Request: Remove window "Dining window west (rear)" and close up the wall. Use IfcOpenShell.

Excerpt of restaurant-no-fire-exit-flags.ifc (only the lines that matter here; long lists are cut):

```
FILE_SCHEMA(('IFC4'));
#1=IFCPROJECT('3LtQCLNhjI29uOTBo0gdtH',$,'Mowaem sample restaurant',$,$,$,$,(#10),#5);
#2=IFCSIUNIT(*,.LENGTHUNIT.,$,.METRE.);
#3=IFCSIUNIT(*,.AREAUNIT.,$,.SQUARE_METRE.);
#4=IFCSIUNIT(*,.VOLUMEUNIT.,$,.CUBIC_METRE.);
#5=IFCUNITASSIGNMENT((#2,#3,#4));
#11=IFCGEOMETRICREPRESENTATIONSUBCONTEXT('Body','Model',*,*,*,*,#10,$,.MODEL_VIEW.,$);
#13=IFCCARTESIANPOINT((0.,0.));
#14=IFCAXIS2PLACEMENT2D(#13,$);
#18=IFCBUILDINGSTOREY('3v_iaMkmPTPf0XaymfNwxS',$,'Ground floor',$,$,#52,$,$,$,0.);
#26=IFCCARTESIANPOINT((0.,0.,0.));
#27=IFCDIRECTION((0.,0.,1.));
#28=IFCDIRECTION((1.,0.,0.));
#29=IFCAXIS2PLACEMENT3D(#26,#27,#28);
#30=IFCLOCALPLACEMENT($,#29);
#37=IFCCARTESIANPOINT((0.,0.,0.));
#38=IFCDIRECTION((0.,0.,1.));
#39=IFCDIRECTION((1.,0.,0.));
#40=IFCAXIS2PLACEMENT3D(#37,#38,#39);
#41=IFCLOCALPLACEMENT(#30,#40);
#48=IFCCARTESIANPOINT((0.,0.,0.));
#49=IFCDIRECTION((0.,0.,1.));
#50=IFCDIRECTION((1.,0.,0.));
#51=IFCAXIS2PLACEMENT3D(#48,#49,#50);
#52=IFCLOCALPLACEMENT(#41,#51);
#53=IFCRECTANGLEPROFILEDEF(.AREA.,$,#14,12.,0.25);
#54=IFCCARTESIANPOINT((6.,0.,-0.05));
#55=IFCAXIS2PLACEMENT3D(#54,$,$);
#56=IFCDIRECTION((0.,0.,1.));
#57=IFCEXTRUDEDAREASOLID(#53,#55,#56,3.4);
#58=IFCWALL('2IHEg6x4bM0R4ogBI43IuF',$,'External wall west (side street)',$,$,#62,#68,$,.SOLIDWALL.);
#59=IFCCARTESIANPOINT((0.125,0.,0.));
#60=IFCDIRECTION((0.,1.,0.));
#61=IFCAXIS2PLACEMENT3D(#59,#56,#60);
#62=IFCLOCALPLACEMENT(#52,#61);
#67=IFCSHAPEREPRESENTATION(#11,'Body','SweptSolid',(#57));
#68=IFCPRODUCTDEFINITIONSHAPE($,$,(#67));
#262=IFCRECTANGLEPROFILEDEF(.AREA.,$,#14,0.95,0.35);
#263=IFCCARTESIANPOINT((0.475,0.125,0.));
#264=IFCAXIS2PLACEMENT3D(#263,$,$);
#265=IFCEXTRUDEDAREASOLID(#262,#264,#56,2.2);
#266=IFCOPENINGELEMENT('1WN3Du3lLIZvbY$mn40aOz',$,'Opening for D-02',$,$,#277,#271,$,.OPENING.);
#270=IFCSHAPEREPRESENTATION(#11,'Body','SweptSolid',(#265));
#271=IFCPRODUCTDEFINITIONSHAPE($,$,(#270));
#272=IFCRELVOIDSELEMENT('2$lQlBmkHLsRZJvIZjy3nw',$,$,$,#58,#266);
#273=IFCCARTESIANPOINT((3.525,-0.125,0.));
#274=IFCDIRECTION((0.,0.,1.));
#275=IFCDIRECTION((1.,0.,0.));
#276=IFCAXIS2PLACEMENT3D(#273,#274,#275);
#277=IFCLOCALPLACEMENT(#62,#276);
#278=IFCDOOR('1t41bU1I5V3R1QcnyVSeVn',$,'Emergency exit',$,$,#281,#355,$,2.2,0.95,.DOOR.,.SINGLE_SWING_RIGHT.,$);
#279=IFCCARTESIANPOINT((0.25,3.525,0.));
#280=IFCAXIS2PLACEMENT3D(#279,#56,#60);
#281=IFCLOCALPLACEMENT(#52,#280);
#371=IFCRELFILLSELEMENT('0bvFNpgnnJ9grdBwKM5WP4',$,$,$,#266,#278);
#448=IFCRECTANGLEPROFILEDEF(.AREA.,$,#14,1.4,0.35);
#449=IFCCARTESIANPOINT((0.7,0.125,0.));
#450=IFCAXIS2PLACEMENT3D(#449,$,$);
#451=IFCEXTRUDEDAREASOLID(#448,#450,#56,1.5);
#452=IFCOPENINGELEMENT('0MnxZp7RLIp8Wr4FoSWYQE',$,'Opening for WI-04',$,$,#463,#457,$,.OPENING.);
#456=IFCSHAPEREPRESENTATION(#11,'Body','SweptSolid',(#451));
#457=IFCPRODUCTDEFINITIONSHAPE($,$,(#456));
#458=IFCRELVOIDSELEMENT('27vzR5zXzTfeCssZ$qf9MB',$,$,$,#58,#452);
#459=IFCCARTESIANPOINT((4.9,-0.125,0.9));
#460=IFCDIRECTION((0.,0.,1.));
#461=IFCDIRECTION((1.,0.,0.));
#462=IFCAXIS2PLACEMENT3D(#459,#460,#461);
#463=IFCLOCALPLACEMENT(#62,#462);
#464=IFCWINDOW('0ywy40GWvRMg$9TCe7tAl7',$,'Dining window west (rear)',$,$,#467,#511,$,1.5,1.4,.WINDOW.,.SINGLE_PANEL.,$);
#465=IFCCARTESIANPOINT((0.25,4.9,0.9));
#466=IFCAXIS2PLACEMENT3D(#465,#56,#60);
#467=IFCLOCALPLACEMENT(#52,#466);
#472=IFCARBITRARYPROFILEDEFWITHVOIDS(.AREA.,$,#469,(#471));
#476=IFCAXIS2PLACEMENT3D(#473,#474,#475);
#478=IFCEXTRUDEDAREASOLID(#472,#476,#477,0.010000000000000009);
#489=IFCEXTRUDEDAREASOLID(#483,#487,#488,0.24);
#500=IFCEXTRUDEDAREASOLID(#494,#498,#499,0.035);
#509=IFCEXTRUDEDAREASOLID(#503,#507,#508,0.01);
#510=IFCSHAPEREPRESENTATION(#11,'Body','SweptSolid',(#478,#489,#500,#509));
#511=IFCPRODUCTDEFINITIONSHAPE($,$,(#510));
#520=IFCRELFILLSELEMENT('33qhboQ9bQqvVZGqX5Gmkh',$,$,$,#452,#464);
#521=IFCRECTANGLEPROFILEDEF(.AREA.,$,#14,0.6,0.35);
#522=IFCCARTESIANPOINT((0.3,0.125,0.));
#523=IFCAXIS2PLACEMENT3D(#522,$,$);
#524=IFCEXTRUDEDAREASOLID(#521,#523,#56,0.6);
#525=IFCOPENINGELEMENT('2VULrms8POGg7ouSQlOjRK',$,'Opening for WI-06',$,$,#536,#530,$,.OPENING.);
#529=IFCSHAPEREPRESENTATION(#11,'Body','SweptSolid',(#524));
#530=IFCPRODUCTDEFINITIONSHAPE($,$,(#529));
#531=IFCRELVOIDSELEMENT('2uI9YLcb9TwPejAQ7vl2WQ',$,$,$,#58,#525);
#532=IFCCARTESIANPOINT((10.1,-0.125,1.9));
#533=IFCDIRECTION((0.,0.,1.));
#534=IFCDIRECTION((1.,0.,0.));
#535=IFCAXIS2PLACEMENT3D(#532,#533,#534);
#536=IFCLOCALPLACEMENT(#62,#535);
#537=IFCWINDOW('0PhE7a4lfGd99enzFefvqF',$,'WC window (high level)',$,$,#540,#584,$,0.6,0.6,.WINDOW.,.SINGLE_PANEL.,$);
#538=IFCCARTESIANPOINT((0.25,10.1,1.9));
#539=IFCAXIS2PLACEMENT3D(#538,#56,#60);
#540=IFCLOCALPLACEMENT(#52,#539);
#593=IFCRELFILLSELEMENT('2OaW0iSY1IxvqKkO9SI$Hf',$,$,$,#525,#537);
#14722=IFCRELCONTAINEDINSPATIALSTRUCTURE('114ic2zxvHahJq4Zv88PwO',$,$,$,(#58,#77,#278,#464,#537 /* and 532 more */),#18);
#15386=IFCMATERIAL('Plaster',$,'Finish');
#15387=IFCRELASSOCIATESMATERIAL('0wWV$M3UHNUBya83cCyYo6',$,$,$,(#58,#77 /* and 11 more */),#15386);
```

```python
import ifcopenshell
import ifcopenshell.api.feature
import ifcopenshell.api.root
import ifcopenshell.geom
import ifcopenshell.util.shape

model = ifcopenshell.open("restaurant-no-fire-exit-flags.ifc")
settings = ifcopenshell.geom.settings()


def volume(element):
    """Net volume in cubic metres, openings subtracted."""
    shape = ifcopenshell.geom.create_shape(settings, element)
    return ifcopenshell.util.shape.get_volume(shape.geometry)


window = model.by_guid("0ywy40GWvRMg$9TCe7tAl7")
opening = window.FillsVoids[0].RelatingOpeningElement
wall = opening.VoidsElements[0].RelatingBuildingElement
before = volume(wall)

ifcopenshell.api.root.remove_product(model, product=window)
ifcopenshell.api.feature.remove_feature(model, feature=opening)

after = volume(wall)

print(f"wall volume {before:.3f} -> {after:.3f} m3")

model.write("restaurant-no-fire-exit-flags_rev.ifc")
```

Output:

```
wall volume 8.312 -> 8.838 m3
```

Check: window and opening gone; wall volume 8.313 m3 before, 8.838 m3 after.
